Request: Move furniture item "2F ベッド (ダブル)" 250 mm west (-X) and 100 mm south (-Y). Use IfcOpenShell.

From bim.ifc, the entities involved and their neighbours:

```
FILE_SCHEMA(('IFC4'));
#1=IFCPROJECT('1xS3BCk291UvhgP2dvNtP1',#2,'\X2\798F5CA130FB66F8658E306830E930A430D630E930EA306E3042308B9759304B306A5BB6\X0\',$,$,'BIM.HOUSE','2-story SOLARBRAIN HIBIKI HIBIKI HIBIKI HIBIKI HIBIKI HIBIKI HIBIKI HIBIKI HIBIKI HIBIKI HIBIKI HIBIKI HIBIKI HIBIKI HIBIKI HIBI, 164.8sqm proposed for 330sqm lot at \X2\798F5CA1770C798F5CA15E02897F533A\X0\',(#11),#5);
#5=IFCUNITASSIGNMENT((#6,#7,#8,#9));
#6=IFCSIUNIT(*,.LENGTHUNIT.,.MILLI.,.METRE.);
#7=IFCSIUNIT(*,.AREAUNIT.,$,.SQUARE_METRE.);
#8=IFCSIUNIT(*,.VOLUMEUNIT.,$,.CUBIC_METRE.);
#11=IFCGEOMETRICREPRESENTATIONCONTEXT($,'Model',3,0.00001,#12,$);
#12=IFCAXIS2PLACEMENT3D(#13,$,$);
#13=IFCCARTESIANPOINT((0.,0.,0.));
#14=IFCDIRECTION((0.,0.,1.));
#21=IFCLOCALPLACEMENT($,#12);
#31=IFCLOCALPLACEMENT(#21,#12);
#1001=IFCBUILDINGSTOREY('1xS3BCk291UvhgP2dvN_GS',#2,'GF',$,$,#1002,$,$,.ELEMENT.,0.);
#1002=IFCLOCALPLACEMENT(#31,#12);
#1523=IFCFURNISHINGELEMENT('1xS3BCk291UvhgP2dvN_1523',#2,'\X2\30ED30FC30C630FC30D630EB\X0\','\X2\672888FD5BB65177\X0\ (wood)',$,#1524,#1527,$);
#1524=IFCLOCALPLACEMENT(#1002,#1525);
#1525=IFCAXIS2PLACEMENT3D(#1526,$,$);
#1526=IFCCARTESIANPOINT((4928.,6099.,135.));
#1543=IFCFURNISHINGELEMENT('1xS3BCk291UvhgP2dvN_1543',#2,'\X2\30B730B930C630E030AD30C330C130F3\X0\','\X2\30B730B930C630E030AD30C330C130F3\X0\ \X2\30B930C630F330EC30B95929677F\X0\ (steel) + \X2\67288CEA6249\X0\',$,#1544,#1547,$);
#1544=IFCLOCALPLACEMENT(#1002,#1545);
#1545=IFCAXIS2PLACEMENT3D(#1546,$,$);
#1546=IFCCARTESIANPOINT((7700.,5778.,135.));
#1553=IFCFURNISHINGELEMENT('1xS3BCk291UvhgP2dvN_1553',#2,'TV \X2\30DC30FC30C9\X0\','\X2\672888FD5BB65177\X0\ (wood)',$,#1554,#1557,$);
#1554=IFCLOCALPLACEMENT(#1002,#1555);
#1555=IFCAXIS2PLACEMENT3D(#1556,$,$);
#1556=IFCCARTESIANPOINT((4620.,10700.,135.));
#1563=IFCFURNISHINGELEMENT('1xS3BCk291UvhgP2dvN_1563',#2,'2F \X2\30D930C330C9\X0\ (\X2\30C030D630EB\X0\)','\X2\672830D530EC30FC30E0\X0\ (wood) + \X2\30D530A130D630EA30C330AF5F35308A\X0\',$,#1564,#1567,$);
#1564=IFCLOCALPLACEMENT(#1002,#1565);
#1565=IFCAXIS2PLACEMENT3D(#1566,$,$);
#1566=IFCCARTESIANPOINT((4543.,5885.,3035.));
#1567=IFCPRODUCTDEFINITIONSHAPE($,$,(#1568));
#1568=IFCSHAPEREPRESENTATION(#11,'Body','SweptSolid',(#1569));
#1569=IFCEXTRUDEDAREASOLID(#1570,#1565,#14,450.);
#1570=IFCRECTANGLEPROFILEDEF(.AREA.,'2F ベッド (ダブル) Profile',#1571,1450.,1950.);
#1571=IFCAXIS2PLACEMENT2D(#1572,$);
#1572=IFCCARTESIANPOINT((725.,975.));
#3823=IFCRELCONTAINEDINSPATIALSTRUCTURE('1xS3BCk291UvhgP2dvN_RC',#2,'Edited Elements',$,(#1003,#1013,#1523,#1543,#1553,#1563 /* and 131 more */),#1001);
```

```python
import ifcopenshell
import ifcopenshell.api.geometry
import ifcopenshell.util.placement
import ifcopenshell.util.unit

model = ifcopenshell.open("bim.ifc")
unit_scale = ifcopenshell.util.unit.calculate_unit_scale(model)

item = model.by_guid("1xS3BCk291UvhgP2dvN_1563")
matrix = ifcopenshell.util.placement.get_local_placement(item.ObjectPlacement)
matrix[0, 3] -= 0.25 / unit_scale
matrix[1, 3] -= 0.1 / unit_scale
ifcopenshell.api.geometry.edit_object_placement(model, product=item, matrix=matrix, is_si=False)

print(ifcopenshell.util.placement.get_local_placement(item.ObjectPlacement).round(3) + 0.0)

model.write("bim_rev.ifc")
```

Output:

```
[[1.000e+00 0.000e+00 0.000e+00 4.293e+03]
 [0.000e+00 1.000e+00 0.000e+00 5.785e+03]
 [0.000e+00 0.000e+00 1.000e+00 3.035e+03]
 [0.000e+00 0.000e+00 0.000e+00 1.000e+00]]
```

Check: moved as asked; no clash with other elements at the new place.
